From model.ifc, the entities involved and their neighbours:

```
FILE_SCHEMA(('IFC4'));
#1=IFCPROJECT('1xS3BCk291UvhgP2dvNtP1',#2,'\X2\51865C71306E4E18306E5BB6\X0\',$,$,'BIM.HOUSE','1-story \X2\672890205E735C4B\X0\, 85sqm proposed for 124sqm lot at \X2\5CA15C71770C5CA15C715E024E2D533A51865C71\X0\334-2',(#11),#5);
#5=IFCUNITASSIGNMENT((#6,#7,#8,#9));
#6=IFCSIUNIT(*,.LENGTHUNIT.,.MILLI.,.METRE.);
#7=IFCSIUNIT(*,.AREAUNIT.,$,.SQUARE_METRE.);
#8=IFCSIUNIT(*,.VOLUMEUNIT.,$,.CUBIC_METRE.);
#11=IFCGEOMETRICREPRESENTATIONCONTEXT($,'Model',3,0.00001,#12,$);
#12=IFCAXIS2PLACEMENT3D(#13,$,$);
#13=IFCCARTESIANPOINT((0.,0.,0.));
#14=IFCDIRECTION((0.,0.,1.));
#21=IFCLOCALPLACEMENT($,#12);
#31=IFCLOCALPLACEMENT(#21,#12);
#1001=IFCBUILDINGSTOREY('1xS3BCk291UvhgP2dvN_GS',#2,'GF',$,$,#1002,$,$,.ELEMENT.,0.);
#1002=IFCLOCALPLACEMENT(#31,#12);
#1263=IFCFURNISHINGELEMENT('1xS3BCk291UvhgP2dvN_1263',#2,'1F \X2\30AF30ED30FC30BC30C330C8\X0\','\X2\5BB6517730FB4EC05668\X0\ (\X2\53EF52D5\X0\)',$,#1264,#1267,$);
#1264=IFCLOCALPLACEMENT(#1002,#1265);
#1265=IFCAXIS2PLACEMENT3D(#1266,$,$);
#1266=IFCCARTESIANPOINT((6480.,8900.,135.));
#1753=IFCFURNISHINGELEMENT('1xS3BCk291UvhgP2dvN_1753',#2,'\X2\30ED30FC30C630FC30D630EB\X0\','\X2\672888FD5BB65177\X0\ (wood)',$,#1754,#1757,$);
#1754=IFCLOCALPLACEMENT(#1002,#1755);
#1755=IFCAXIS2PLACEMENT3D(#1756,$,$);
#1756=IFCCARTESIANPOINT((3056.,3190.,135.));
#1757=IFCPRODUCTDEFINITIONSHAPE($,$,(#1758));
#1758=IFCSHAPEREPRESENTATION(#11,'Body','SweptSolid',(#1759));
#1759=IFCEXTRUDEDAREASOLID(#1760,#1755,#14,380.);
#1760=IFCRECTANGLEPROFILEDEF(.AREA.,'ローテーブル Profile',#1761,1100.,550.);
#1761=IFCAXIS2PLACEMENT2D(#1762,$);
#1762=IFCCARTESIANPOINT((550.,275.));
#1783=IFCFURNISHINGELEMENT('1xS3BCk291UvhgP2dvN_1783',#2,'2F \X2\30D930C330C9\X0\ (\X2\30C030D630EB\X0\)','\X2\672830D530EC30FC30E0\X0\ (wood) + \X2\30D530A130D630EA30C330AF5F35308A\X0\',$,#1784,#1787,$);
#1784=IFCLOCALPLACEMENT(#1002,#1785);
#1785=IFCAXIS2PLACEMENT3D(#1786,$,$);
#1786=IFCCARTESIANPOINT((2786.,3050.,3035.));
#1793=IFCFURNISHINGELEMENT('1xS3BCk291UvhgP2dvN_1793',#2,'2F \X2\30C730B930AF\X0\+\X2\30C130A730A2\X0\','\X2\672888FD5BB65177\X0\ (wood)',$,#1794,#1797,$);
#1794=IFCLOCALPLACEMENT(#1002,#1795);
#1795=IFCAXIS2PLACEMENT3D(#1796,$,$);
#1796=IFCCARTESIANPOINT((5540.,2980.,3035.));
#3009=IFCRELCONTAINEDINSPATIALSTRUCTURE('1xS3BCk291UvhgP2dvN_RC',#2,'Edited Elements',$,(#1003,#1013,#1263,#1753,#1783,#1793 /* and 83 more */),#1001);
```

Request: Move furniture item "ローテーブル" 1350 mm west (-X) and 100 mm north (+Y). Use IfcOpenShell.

```python
import ifcopenshell
import ifcopenshell.api.geometry
import ifcopenshell.util.placement
import ifcopenshell.util.unit

model = ifcopenshell.open("model.ifc")
unit_scale = ifcopenshell.util.unit.calculate_unit_scale(model)

item = model.by_id(1753)
matrix = ifcopenshell.util.placement.get_local_placement(item.ObjectPlacement)
matrix[0, 3] -= 1.35 / unit_scale
matrix[1, 3] += 0.1 / unit_scale
ifcopenshell.api.geometry.edit_object_placement(model, product=item, matrix=matrix, is_si=False)

print(ifcopenshell.util.placement.get_local_placement(item.ObjectPlacement).round(3) + 0.0)

model.write("model_rev.ifc")
```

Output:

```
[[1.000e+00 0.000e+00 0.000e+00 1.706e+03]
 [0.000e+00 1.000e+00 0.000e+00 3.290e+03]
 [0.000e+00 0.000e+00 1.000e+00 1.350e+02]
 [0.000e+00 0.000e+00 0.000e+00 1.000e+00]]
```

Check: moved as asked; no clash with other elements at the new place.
